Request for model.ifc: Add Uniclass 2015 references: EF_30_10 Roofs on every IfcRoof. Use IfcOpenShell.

First a look at what the model holds.

```python
import ifcopenshell

model = ifcopenshell.open("model.ifc")
print(model.schema)
print("classifications:", [c.Name for c in model.by_type("IfcClassification")])
for ifc_class in ("IfcDoor", "IfcRoof", "IfcStair", "IfcWall", "IfcWindow"):
    print(ifc_class, len(model.by_type(ifc_class)))
```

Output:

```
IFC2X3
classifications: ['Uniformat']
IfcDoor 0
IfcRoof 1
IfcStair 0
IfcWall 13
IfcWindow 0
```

```python
import ifcopenshell
import ifcopenshell.api.classification

model = ifcopenshell.open("model.ifc")

# IFC2X3 requires Source and Edition and has no link from the project to the system.
system = model.create_entity("IfcClassification", Source="NBS", Edition="2015", Name="Uniclass 2015")

codes = {
    "IfcRoof": ("EF_30_10", "Roofs"),
}
for ifc_class, (code, name) in codes.items():
    products = model.by_type(ifc_class)
    ifcopenshell.api.classification.add_reference(
        model, products=products, classification=system, identification=code, name=name
    )
    print(code, len(products))

model.write("model_updated.ifc")
```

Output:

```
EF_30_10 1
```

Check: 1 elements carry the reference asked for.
